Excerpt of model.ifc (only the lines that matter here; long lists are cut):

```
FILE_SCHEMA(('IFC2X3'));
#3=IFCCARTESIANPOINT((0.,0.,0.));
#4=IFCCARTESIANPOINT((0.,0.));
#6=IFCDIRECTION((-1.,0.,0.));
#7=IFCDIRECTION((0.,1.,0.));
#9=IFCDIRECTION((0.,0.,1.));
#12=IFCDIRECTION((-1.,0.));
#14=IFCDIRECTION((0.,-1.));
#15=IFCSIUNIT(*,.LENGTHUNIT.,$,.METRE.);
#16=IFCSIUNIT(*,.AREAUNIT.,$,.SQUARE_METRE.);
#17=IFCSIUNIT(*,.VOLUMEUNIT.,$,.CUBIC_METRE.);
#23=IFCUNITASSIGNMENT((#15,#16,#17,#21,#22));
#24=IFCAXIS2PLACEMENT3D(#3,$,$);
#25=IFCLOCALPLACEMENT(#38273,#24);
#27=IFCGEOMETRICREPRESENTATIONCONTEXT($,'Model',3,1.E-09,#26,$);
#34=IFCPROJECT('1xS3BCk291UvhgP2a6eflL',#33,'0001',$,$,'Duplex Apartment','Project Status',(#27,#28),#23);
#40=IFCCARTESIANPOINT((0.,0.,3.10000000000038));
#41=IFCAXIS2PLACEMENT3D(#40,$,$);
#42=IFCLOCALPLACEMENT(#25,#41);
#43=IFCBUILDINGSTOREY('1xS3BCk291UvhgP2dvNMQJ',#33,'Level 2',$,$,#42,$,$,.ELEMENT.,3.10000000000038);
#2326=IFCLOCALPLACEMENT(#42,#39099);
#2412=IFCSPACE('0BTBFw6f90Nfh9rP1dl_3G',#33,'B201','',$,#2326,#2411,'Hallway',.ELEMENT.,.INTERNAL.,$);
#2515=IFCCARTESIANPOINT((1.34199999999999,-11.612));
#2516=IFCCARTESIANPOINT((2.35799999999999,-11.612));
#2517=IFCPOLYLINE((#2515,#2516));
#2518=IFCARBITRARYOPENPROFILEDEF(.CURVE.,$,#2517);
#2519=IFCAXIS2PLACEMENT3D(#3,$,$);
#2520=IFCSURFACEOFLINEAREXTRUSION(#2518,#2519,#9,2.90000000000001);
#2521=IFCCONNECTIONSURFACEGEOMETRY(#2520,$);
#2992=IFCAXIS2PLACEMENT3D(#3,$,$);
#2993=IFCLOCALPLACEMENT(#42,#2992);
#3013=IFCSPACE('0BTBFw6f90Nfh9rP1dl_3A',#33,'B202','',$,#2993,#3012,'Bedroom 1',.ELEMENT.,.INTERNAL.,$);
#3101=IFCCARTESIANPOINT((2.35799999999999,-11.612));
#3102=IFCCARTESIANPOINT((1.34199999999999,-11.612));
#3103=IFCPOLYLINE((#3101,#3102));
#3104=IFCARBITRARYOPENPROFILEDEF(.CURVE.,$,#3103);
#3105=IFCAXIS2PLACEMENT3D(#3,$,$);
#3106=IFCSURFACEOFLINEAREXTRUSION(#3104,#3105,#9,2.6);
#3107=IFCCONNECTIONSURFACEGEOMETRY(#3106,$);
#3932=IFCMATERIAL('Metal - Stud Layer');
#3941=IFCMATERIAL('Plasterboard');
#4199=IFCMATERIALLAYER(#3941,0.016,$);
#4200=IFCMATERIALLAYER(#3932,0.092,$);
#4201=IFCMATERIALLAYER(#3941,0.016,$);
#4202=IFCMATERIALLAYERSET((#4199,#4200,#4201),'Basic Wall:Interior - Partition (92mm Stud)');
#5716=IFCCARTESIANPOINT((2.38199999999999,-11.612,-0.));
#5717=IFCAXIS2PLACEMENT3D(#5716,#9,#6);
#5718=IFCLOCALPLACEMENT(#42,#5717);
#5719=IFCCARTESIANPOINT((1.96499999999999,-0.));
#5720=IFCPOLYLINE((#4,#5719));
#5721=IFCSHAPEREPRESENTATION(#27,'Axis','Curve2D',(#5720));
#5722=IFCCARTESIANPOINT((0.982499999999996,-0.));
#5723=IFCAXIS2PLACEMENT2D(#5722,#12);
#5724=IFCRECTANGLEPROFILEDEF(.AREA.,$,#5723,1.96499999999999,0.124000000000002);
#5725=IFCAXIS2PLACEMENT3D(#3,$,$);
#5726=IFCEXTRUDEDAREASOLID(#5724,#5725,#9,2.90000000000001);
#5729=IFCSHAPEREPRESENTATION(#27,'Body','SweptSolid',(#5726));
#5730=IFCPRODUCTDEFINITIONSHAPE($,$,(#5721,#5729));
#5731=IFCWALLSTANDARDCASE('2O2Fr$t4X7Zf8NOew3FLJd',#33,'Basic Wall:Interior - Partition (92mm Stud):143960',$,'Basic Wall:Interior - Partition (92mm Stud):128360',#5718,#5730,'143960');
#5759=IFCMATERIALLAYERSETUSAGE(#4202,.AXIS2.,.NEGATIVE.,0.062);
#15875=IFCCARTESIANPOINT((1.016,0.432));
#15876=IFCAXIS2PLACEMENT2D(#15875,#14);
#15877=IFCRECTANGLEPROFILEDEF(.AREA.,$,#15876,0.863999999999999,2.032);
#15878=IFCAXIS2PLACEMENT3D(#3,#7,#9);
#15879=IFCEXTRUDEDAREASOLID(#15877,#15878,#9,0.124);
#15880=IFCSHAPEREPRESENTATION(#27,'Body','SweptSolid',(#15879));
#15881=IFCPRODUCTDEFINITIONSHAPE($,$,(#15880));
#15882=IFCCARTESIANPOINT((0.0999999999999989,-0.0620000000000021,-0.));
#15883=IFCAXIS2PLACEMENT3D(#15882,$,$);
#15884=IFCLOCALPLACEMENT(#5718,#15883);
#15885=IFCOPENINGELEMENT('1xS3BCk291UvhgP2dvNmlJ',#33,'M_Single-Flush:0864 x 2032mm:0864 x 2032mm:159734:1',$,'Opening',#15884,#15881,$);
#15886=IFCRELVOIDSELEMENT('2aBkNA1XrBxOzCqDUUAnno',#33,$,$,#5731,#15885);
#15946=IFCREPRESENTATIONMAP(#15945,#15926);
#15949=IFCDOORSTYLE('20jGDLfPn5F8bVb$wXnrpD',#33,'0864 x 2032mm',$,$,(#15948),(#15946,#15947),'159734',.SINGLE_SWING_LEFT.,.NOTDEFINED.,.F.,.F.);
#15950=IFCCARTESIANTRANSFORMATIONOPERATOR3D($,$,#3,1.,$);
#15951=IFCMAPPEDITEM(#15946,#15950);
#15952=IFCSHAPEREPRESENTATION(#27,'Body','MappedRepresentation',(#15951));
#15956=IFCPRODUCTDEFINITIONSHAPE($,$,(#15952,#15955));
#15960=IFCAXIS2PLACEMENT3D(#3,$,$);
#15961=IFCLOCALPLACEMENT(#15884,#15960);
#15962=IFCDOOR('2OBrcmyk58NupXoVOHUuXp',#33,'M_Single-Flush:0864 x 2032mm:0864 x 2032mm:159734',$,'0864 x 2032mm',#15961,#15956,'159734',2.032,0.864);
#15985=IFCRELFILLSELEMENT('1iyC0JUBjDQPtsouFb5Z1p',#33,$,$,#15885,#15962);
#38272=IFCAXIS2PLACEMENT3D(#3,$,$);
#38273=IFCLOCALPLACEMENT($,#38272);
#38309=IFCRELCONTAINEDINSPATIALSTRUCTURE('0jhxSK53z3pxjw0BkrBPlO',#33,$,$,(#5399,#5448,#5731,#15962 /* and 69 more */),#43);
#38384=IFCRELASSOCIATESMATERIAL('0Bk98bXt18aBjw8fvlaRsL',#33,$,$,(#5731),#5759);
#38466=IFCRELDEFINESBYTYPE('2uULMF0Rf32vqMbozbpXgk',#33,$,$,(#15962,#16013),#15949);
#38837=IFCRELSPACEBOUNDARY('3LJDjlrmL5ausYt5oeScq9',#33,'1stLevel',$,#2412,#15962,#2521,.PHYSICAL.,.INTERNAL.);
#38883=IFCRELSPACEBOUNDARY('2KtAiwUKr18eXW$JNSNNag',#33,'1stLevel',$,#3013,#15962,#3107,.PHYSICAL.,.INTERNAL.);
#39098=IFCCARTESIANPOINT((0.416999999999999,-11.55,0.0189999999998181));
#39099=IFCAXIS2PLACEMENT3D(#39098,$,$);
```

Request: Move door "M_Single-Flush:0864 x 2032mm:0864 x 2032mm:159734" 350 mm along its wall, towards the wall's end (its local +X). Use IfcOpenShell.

```python
import numpy as np
import ifcopenshell
import ifcopenshell.api.geometry
import ifcopenshell.util.placement

model = ifcopenshell.open("model.ifc")

door = model.by_guid("2OBrcmyk58NupXoVOHUuXp")
opening = door.FillsVoids[0].RelatingOpeningElement
wall = opening.VoidsElements[0].RelatingBuildingElement

wall_matrix = ifcopenshell.util.placement.get_local_placement(wall.ObjectPlacement)
shift = wall_matrix[:3, 0] * 0.35
before = ifcopenshell.util.placement.get_local_placement(door.ObjectPlacement)[:3, 3].copy()

# The door is placed relative to its opening, so it follows when the opening moves.
matrix = ifcopenshell.util.placement.get_local_placement(opening.ObjectPlacement)
matrix[:3, 3] += shift
ifcopenshell.api.geometry.edit_object_placement(
    model, product=opening, matrix=matrix, is_si=False, should_transform_children=True
)

# Space boundary surfaces are stored in each space's coordinates; move them too.
for rel in door.ProvidesBoundaries:
    if not rel.ConnectionGeometry:
        continue
    surface = rel.ConnectionGeometry.SurfaceOnRelatingElement
    space_matrix = ifcopenshell.util.placement.get_local_placement(rel.RelatingSpace.ObjectPlacement)
    point = np.array(surface.Position.Location.Coordinates) + space_matrix[:3, :3].T @ shift
    surface.Position = model.createIfcAxis2Placement3D(
        model.createIfcCartesianPoint(point.tolist()), surface.Position.Axis, surface.Position.RefDirection
    )

after = ifcopenshell.util.placement.get_local_placement(door.ObjectPlacement)[:3, 3]
print("door moved by", (after - before).round(3) + 0.0)

model.write("model_rev.ifc")
```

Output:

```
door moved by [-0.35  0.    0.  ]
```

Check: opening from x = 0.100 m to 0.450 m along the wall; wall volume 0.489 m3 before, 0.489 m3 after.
